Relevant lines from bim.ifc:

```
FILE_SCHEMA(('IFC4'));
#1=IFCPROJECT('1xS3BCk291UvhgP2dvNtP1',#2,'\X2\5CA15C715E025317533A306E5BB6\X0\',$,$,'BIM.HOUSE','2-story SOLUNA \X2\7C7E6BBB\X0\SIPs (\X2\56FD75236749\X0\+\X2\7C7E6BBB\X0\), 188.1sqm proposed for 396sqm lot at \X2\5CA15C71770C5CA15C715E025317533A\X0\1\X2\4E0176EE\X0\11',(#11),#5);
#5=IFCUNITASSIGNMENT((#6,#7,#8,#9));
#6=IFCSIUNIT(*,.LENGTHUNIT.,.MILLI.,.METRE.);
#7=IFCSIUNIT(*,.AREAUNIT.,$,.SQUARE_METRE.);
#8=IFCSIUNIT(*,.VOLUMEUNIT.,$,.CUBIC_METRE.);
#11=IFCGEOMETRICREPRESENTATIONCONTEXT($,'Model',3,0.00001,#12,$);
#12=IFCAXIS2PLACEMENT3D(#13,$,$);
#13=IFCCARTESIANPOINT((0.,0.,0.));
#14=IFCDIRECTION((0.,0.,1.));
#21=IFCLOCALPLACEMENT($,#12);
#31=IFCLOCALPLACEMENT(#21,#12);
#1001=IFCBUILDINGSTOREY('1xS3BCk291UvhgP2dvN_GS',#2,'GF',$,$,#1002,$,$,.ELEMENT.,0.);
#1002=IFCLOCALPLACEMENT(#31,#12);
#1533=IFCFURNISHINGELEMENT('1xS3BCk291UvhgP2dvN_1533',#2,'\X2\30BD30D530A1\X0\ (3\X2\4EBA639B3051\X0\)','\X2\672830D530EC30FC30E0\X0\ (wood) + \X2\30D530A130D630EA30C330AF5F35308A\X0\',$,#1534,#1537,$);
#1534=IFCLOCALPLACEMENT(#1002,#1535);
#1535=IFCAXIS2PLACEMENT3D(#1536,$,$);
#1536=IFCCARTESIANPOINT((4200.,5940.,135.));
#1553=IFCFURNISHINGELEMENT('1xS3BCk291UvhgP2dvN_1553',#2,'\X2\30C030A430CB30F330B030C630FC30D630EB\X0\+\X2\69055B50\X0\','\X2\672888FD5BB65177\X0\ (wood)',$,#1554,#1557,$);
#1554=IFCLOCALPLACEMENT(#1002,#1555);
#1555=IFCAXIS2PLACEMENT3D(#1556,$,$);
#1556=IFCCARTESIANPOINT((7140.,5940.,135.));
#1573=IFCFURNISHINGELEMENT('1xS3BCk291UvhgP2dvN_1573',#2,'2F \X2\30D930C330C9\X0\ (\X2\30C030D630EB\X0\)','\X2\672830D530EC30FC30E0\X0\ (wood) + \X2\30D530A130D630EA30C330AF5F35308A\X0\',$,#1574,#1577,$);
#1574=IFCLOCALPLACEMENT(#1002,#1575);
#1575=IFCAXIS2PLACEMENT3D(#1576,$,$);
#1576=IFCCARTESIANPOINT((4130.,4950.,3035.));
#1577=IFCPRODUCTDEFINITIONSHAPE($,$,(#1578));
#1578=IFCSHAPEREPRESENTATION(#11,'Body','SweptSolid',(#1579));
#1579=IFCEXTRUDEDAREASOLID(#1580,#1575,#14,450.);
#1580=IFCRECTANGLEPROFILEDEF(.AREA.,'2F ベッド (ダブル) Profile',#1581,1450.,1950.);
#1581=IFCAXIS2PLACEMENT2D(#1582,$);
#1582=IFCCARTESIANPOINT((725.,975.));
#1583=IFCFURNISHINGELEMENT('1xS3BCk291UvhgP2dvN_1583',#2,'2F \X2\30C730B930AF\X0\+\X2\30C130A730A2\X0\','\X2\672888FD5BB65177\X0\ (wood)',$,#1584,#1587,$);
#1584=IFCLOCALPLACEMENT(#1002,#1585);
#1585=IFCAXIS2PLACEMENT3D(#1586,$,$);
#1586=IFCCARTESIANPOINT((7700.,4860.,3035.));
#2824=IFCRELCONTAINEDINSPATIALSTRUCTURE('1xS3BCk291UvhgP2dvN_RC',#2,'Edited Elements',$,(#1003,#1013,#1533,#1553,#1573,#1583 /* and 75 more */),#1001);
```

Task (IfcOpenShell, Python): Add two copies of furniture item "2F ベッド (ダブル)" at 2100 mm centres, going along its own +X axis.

```python
import ifcopenshell
import ifcopenshell.api.geometry
import ifcopenshell.api.root
import ifcopenshell.util.element
import ifcopenshell.util.placement

model = ifcopenshell.open("bim.ifc")


def reuse_history(source, copy):
    """copy_class also copies each property set's owner history, people and application; keep the originals."""
    for rel in copy.IsDefinedBy:
        if rel.is_a("IfcRelDefinesByProperties") and (history := rel.RelatingPropertyDefinition.OwnerHistory):
            rel.RelatingPropertyDefinition.OwnerHistory = source.OwnerHistory
            ifcopenshell.util.element.remove_deep2(model, history)


source = model.by_guid("1xS3BCk291UvhgP2dvN_1573")
base = ifcopenshell.util.placement.get_local_placement(source.ObjectPlacement)
step = base[:3, 0] * 2100.0

for i in range(1, 3):
    copy = ifcopenshell.api.root.copy_class(model, product=source)
    copy.Representation = ifcopenshell.util.element.copy_deep(
        model, source.Representation, exclude=["IfcGeometricRepresentationContext", "IfcRepresentationMap"]
    )
    reuse_history(source, copy)
    matrix = base.copy()
    matrix[:3, 3] += i * step
    print("added at", matrix[:3, 3].round(3) + 0.0)
    ifcopenshell.api.geometry.edit_object_placement(model, product=copy, matrix=matrix, is_si=False)

model.write("bim-out.ifc")
```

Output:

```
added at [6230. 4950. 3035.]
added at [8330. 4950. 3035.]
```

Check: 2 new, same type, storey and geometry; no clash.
